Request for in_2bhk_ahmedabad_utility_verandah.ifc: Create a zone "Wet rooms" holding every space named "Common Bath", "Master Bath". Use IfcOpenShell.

First a look at what the model holds.

```python
import ifcopenshell

model = ifcopenshell.open("in_2bhk_ahmedabad_utility_verandah.ifc")
print(model.schema)
seen = {}
for space in model.by_type("IfcSpace"):
    seen[space.LongName] = seen.get(space.LongName, 0) + 1
for name, count in sorted(seen.items(), key=str):
    print(count, "x", name)
print("zones:", [z.Name for z in model.by_type("IfcZone")][:20])
```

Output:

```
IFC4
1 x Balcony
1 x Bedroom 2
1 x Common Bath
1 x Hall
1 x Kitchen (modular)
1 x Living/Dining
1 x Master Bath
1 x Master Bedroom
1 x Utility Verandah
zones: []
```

```python
import ifcopenshell
import ifcopenshell.api.group
import ifcopenshell.api.root

model = ifcopenshell.open("in_2bhk_ahmedabad_utility_verandah.ifc")

names = {"Common Bath", "Master Bath"}
spaces = [s for s in model.by_type("IfcSpace") if s.LongName in names]

zone = ifcopenshell.api.root.create_entity(model, ifc_class="IfcZone", name="Wet rooms")
ifcopenshell.api.group.assign_group(model, products=spaces, group=zone)
print(len(spaces), "spaces in", zone.Name)

model.write("in_2bhk_ahmedabad_utility_verandah-out.ifc")
```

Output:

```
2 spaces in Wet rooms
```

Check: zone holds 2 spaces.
